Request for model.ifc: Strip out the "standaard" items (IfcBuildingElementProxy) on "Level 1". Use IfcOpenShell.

First a look at what the model holds.

```python
import ifcopenshell
import ifcopenshell.util.element

model = ifcopenshell.open("model.ifc")
print(model.schema)
storey = next(s for s in model.by_type("IfcBuildingStorey") if s.Name == "Level 1")
proxies = [e for e in ifcopenshell.util.element.get_decomposition(storey) if e.is_a("IfcBuildingElementProxy")]
seen = {}
for e in proxies:
    element_type = ifcopenshell.util.element.get_type(e)
    name = element_type.Name if element_type not in (None, e) else None
    seen[name] = seen.get(name, 0) + 1
for name, count in sorted(seen.items(), key=str):
    print(count, "x", name)
```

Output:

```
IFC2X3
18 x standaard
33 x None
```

```python
import ifcopenshell
import ifcopenshell.api.root
import ifcopenshell.util.element

model = ifcopenshell.open("model.ifc")

storey = next(s for s in model.by_type("IfcBuildingStorey") if s.Name == "Level 1")
proxies = [e for e in ifcopenshell.util.element.get_decomposition(storey) if e.is_a("IfcBuildingElementProxy")]
targets = [e for e in proxies if (t := ifcopenshell.util.element.get_type(e)) not in (None, e) and t.Name == "standaard"]

for e in targets:
    ifcopenshell.api.root.remove_product(model, product=e)
print(len(targets), "removed")

model.write("model_updated.ifc")
```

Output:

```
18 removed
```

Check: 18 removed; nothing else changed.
